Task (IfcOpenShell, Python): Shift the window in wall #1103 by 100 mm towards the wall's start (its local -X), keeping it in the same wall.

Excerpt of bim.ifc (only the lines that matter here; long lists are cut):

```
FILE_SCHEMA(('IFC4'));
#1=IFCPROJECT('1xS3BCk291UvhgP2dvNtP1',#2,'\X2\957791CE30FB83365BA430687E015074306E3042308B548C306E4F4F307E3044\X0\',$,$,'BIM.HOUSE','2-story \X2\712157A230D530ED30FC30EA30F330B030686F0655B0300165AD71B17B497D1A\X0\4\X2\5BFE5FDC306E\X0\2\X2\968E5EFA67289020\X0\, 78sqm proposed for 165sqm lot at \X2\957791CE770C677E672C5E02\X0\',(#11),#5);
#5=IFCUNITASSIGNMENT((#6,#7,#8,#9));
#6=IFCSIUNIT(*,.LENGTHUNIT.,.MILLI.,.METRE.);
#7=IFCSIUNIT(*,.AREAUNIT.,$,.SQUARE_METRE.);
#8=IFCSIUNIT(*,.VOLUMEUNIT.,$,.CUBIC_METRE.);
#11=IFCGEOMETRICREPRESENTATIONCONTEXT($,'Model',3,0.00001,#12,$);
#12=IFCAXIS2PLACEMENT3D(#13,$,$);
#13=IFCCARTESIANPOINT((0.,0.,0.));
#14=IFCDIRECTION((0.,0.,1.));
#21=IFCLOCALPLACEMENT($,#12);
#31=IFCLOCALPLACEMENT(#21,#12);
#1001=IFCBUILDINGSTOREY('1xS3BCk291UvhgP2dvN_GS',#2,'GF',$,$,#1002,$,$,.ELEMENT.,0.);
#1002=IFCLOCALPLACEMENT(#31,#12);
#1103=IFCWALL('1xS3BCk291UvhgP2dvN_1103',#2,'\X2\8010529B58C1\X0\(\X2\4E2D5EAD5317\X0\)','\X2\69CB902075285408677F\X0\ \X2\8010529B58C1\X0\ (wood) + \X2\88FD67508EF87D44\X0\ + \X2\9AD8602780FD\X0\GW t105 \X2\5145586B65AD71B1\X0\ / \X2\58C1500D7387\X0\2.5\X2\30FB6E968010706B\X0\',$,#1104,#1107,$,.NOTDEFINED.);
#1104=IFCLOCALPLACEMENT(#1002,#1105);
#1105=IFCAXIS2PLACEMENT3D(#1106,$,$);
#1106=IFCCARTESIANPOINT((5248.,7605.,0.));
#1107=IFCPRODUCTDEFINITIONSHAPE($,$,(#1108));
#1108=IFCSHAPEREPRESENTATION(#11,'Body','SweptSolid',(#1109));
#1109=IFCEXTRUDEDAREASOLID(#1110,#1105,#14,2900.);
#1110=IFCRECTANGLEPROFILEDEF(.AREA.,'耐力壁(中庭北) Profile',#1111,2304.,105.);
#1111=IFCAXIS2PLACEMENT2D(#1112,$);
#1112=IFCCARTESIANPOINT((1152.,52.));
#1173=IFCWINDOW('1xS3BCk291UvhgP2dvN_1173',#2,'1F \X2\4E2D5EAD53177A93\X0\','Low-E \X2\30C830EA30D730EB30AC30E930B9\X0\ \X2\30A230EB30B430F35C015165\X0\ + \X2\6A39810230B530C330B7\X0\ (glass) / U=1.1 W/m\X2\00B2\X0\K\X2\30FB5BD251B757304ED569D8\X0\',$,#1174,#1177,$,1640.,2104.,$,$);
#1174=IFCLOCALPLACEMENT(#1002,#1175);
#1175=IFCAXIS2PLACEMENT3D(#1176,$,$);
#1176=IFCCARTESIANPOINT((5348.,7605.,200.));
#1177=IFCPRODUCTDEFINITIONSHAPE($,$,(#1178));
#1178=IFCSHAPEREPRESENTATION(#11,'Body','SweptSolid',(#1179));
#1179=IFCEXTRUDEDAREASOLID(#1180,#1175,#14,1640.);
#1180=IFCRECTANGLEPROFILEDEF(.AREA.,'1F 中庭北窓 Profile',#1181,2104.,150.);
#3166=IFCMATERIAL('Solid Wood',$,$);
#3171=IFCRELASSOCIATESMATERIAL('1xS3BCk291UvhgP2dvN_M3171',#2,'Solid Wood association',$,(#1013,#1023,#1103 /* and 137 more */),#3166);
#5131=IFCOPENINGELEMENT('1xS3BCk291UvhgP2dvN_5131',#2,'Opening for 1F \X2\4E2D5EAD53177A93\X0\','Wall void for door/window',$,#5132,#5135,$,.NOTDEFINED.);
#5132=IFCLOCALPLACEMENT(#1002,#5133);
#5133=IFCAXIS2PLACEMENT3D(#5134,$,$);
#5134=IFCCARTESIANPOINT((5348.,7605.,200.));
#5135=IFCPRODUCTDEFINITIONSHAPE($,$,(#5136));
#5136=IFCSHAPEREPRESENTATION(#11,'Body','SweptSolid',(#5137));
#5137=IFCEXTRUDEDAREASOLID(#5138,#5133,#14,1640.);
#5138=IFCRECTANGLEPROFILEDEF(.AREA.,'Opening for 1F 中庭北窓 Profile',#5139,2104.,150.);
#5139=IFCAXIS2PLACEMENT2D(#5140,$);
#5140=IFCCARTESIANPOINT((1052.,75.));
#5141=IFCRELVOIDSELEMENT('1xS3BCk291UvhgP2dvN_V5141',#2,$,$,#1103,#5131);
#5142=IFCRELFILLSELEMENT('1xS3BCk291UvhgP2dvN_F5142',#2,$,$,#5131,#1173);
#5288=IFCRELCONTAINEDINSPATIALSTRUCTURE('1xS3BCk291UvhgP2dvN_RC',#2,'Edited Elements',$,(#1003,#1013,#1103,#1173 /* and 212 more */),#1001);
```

```python
import ifcopenshell
import ifcopenshell.api.geometry
import ifcopenshell.util.placement

model = ifcopenshell.open("bim.ifc")

window = model.by_guid("1xS3BCk291UvhgP2dvN_1173")
opening = window.FillsVoids[0].RelatingOpeningElement
wall = opening.VoidsElements[0].RelatingBuildingElement

wall_matrix = ifcopenshell.util.placement.get_local_placement(wall.ObjectPlacement)
shift = wall_matrix[:3, 0] * -100.0
before = ifcopenshell.util.placement.get_local_placement(window.ObjectPlacement)[:3, 3].copy()

# The window is not placed relative to its opening, so move both.
for product in (opening, window):
    matrix = ifcopenshell.util.placement.get_local_placement(product.ObjectPlacement)
    matrix[:3, 3] += shift
    ifcopenshell.api.geometry.edit_object_placement(model, product=product, matrix=matrix, is_si=False)

after = ifcopenshell.util.placement.get_local_placement(window.ObjectPlacement)[:3, 3]
print("window moved by", (after - before).round(3) + 0.0)

model.write("bim_edited.ifc")
```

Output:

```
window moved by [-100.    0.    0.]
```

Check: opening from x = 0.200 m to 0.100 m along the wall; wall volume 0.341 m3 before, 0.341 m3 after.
